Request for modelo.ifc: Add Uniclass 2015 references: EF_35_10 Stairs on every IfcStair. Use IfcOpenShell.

First a look at what the model holds.

```python
import ifcopenshell

model = ifcopenshell.open("modelo.ifc")
print(model.schema)
print("classifications:", [c.Name for c in model.by_type("IfcClassification")])
for ifc_class in ("IfcDoor", "IfcRoof", "IfcStair", "IfcWall", "IfcWindow"):
    print(ifc_class, len(model.by_type(ifc_class)))
```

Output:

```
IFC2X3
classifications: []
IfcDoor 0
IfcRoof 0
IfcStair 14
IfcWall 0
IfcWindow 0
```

```python
import ifcopenshell
import ifcopenshell.api.classification

model = ifcopenshell.open("modelo.ifc")

# IFC2X3 requires Source and Edition and has no link from the project to the system.
system = model.create_entity("IfcClassification", Source="NBS", Edition="2015", Name="Uniclass 2015")

codes = {
    "IfcStair": ("EF_35_10", "Stairs"),
}
for ifc_class, (code, name) in codes.items():
    products = model.by_type(ifc_class)
    ifcopenshell.api.classification.add_reference(
        model, products=products, classification=system, identification=code, name=name
    )
    print(code, len(products))

model.write("modelo_rev.ifc")
```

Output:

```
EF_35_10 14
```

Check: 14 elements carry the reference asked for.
